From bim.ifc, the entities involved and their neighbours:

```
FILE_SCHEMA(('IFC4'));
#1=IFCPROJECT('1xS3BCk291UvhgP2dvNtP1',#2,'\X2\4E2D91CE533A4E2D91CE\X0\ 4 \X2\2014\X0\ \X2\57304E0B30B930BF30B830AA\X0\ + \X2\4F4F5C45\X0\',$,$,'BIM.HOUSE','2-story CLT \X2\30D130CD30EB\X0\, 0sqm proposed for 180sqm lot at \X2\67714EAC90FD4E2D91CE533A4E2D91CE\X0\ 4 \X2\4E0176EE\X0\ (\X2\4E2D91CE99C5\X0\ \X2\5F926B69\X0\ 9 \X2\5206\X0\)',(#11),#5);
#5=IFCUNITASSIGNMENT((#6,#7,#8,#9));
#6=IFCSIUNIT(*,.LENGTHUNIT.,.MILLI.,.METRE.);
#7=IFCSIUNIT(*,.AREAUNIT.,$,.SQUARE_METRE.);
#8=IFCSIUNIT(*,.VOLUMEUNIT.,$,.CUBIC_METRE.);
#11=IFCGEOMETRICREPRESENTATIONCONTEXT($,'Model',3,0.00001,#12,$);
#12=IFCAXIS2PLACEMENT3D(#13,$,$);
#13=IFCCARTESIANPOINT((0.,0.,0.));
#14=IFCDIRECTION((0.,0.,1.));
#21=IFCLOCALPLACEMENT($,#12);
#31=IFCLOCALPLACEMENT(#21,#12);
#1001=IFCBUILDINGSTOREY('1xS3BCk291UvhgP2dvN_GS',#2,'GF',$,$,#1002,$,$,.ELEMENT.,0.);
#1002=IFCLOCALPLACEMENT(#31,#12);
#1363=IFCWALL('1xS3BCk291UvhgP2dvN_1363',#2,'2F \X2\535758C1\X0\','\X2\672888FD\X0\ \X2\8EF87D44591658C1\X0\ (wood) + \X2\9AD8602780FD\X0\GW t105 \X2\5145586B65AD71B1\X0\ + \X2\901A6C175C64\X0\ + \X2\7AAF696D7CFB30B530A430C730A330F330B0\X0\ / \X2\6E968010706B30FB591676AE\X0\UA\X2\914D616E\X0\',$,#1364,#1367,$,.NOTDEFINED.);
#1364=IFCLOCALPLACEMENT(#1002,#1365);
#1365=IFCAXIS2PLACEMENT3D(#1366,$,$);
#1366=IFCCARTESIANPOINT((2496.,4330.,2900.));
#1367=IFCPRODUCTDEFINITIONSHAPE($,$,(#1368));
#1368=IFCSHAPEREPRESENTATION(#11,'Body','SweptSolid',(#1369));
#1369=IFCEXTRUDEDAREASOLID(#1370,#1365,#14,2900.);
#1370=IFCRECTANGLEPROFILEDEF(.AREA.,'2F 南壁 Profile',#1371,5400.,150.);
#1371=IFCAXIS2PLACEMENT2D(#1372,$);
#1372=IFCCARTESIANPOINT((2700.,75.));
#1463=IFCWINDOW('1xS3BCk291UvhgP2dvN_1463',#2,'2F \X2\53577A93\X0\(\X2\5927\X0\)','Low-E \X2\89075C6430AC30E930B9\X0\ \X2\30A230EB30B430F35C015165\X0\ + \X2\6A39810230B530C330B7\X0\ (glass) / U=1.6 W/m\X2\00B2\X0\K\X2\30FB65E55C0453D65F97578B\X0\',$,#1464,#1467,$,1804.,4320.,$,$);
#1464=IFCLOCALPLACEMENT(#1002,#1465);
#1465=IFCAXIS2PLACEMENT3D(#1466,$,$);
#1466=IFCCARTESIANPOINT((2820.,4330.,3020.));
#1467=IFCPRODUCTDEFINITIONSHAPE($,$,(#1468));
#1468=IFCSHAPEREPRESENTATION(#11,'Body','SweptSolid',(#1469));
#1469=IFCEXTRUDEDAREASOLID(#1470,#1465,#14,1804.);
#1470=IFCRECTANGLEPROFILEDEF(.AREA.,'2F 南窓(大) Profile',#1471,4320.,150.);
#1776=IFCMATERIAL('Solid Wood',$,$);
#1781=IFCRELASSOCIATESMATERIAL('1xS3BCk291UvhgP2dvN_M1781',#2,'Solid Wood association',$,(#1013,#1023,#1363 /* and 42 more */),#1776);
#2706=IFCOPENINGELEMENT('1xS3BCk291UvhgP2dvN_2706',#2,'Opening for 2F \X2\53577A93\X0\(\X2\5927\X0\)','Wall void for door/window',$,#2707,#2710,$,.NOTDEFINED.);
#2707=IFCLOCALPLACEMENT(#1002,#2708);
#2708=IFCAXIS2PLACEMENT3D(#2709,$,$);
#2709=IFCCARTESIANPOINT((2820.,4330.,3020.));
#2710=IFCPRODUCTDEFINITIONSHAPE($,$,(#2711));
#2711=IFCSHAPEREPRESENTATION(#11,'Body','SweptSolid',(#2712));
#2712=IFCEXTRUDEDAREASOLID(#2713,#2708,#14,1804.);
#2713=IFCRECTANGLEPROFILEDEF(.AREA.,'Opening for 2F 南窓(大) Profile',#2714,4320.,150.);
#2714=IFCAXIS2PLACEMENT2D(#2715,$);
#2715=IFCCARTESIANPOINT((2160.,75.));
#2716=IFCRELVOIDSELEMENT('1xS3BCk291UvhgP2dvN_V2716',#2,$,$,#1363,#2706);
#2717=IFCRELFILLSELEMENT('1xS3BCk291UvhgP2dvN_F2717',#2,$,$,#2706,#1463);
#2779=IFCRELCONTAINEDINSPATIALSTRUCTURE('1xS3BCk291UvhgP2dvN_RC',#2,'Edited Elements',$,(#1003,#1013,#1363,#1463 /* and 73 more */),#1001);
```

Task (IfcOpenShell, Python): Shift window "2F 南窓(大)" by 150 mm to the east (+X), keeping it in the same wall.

```python
import ifcopenshell
import ifcopenshell.api.geometry
import ifcopenshell.util.placement
import ifcopenshell.util.unit

model = ifcopenshell.open("bim.ifc")
unit_scale = ifcopenshell.util.unit.calculate_unit_scale(model)

window = model.by_guid("1xS3BCk291UvhgP2dvN_1463")
opening = window.FillsVoids[0].RelatingOpeningElement
wall = opening.VoidsElements[0].RelatingBuildingElement

wall_matrix = ifcopenshell.util.placement.get_local_placement(wall.ObjectPlacement)
shift = wall_matrix[:3, 0] * 0.15 / unit_scale
before = ifcopenshell.util.placement.get_local_placement(window.ObjectPlacement)[:3, 3].copy()

# The window is not placed relative to its opening, so move both.
for product in (opening, window):
    matrix = ifcopenshell.util.placement.get_local_placement(product.ObjectPlacement)
    matrix[:3, 3] += shift
    ifcopenshell.api.geometry.edit_object_placement(model, product=product, matrix=matrix, is_si=False)

after = ifcopenshell.util.placement.get_local_placement(window.ObjectPlacement)[:3, 3]
print("window moved by", (after - before).round(3) + 0.0)

model.write("bim_rev.ifc")
```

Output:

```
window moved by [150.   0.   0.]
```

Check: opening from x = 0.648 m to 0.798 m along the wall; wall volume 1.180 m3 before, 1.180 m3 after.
